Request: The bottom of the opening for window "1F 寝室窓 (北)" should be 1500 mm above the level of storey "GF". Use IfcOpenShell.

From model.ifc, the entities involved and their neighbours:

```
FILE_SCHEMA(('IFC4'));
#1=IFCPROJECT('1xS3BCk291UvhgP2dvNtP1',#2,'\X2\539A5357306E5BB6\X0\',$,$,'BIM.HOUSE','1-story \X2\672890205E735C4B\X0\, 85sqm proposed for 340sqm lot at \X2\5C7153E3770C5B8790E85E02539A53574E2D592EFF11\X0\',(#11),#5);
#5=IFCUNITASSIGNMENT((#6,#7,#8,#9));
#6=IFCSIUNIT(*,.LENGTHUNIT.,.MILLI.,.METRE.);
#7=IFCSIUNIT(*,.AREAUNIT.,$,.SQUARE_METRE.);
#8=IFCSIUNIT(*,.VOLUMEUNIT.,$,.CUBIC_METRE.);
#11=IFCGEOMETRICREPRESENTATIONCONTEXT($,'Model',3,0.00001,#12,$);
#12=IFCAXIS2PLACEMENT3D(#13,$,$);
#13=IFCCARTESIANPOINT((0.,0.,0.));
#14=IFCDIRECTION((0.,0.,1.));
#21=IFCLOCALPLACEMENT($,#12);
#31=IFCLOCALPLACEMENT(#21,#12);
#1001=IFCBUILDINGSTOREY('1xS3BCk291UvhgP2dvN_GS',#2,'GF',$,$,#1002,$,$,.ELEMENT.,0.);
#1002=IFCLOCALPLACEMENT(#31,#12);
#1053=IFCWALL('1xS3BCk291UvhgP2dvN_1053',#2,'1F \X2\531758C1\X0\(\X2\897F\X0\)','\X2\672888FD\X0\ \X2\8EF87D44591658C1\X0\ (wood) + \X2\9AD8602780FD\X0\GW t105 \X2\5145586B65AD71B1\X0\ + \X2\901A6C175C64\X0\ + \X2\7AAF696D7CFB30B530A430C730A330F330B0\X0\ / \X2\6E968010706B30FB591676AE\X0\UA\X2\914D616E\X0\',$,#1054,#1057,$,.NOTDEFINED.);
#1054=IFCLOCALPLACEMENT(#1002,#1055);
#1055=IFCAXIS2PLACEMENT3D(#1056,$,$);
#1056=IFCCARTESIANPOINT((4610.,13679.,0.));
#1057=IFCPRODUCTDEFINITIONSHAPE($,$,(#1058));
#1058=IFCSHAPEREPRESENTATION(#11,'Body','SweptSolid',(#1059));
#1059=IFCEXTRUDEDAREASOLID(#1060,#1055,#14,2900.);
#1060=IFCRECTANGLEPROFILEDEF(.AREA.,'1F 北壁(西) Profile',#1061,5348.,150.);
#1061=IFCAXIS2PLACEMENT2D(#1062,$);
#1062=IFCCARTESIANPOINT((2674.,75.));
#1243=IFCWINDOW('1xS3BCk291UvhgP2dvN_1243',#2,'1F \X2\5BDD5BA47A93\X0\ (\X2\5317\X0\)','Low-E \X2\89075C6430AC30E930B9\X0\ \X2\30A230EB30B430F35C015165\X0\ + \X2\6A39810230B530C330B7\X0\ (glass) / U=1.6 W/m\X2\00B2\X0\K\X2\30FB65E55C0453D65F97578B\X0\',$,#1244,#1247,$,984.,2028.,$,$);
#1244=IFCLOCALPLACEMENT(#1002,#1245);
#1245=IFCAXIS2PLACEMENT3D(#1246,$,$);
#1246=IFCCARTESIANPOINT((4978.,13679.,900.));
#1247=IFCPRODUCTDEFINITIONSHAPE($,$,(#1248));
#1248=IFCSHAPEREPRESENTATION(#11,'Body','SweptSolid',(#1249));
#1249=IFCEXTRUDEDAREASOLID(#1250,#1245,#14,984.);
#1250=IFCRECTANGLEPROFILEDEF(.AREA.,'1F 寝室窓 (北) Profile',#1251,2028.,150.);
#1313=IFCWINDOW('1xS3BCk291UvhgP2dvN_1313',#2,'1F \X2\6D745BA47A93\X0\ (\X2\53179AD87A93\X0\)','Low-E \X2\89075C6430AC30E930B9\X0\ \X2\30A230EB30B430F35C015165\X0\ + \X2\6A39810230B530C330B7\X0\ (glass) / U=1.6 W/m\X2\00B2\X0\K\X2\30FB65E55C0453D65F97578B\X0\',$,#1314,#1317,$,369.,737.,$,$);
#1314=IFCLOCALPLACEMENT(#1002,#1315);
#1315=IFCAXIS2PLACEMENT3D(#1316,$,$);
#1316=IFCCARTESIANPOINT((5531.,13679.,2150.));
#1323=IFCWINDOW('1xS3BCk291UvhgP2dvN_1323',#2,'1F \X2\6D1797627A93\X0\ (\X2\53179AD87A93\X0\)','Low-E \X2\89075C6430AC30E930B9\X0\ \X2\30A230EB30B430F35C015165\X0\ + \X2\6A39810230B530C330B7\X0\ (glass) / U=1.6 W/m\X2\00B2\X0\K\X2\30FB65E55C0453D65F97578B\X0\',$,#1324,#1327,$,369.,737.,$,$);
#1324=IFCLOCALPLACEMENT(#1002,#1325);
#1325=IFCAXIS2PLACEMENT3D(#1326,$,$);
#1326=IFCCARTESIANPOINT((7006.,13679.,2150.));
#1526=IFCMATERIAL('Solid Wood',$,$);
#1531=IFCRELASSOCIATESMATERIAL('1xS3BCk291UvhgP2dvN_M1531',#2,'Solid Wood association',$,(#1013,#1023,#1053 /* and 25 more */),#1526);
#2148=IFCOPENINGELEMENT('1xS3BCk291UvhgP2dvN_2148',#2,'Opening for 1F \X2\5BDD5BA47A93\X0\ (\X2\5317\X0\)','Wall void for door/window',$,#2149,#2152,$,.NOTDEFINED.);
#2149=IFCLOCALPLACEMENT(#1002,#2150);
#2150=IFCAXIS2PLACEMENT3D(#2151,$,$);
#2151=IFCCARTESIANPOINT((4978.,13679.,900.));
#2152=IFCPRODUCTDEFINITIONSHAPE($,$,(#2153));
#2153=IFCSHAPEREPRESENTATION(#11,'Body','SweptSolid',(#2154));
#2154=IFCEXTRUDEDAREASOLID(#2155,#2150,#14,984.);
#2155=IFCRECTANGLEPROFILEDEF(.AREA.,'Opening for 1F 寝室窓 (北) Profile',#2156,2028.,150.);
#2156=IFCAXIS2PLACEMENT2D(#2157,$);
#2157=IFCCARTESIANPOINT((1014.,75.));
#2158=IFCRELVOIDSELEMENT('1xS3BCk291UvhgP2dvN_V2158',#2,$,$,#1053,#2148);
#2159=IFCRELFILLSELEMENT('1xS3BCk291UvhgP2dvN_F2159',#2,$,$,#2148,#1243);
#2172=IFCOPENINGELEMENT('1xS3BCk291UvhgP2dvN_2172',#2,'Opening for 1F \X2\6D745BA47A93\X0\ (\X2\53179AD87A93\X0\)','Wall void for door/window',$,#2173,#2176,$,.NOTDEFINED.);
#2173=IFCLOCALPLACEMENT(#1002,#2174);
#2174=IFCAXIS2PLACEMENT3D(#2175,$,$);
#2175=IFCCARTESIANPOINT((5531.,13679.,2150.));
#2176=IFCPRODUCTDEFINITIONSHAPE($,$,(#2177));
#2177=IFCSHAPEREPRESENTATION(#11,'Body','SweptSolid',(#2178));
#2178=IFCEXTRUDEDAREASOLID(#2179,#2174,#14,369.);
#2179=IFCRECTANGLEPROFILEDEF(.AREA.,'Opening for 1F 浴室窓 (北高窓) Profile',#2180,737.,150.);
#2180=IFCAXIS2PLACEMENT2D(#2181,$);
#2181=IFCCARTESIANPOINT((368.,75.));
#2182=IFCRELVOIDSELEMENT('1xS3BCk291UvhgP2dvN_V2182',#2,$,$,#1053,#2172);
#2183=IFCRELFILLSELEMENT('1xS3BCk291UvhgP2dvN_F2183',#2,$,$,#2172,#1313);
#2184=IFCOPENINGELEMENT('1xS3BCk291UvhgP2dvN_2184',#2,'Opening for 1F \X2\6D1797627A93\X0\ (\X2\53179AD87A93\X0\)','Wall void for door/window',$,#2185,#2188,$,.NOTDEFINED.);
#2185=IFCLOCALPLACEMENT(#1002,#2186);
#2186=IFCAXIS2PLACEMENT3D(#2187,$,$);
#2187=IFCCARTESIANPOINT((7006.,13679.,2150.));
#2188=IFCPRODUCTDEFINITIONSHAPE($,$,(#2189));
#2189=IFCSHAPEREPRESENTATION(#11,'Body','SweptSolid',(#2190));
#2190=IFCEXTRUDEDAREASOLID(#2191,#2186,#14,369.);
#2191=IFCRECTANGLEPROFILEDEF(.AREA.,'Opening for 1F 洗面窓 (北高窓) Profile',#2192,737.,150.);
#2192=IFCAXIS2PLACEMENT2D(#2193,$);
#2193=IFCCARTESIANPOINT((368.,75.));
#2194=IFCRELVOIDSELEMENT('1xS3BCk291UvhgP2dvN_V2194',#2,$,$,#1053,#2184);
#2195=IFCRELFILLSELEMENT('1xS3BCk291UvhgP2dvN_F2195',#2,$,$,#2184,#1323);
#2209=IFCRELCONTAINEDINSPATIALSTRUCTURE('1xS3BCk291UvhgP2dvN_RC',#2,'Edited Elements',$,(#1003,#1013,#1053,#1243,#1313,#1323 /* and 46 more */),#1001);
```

```python
import numpy as np
import ifcopenshell
import ifcopenshell.api.geometry
import ifcopenshell.geom
import ifcopenshell.util.element
import ifcopenshell.util.placement
import ifcopenshell.util.shape
import ifcopenshell.util.unit

model = ifcopenshell.open("model.ifc")
unit_scale = ifcopenshell.util.unit.calculate_unit_scale(model)

window = model.by_id(1243)
opening = window.FillsVoids[0].RelatingOpeningElement
storey = ifcopenshell.util.element.get_container(window, ifc_class="IfcBuildingStorey")
level = ifcopenshell.util.placement.get_local_placement(storey.ObjectPlacement)[2, 3]

# The opening's origin need not be at the sill, so measure its lowest point.
shape = ifcopenshell.geom.create_shape(ifcopenshell.geom.settings(), opening)
bottom = ifcopenshell.util.shape.get_shape_bottom_elevation(shape, shape.geometry) / unit_scale
dz = level + 1.5 / unit_scale - bottom

shift = np.array([0.0, 0.0, dz])
# The window is not placed relative to its opening, so move both.
for product in (opening, window):
    matrix = ifcopenshell.util.placement.get_local_placement(product.ObjectPlacement)
    matrix[:3, 3] += shift
    ifcopenshell.api.geometry.edit_object_placement(model, product=product, matrix=matrix, is_si=False)

print(f"moved by {dz * unit_scale:+.3f} m")

model.write("model_v2.ifc")
```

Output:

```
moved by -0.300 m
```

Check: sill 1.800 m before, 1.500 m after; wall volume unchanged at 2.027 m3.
